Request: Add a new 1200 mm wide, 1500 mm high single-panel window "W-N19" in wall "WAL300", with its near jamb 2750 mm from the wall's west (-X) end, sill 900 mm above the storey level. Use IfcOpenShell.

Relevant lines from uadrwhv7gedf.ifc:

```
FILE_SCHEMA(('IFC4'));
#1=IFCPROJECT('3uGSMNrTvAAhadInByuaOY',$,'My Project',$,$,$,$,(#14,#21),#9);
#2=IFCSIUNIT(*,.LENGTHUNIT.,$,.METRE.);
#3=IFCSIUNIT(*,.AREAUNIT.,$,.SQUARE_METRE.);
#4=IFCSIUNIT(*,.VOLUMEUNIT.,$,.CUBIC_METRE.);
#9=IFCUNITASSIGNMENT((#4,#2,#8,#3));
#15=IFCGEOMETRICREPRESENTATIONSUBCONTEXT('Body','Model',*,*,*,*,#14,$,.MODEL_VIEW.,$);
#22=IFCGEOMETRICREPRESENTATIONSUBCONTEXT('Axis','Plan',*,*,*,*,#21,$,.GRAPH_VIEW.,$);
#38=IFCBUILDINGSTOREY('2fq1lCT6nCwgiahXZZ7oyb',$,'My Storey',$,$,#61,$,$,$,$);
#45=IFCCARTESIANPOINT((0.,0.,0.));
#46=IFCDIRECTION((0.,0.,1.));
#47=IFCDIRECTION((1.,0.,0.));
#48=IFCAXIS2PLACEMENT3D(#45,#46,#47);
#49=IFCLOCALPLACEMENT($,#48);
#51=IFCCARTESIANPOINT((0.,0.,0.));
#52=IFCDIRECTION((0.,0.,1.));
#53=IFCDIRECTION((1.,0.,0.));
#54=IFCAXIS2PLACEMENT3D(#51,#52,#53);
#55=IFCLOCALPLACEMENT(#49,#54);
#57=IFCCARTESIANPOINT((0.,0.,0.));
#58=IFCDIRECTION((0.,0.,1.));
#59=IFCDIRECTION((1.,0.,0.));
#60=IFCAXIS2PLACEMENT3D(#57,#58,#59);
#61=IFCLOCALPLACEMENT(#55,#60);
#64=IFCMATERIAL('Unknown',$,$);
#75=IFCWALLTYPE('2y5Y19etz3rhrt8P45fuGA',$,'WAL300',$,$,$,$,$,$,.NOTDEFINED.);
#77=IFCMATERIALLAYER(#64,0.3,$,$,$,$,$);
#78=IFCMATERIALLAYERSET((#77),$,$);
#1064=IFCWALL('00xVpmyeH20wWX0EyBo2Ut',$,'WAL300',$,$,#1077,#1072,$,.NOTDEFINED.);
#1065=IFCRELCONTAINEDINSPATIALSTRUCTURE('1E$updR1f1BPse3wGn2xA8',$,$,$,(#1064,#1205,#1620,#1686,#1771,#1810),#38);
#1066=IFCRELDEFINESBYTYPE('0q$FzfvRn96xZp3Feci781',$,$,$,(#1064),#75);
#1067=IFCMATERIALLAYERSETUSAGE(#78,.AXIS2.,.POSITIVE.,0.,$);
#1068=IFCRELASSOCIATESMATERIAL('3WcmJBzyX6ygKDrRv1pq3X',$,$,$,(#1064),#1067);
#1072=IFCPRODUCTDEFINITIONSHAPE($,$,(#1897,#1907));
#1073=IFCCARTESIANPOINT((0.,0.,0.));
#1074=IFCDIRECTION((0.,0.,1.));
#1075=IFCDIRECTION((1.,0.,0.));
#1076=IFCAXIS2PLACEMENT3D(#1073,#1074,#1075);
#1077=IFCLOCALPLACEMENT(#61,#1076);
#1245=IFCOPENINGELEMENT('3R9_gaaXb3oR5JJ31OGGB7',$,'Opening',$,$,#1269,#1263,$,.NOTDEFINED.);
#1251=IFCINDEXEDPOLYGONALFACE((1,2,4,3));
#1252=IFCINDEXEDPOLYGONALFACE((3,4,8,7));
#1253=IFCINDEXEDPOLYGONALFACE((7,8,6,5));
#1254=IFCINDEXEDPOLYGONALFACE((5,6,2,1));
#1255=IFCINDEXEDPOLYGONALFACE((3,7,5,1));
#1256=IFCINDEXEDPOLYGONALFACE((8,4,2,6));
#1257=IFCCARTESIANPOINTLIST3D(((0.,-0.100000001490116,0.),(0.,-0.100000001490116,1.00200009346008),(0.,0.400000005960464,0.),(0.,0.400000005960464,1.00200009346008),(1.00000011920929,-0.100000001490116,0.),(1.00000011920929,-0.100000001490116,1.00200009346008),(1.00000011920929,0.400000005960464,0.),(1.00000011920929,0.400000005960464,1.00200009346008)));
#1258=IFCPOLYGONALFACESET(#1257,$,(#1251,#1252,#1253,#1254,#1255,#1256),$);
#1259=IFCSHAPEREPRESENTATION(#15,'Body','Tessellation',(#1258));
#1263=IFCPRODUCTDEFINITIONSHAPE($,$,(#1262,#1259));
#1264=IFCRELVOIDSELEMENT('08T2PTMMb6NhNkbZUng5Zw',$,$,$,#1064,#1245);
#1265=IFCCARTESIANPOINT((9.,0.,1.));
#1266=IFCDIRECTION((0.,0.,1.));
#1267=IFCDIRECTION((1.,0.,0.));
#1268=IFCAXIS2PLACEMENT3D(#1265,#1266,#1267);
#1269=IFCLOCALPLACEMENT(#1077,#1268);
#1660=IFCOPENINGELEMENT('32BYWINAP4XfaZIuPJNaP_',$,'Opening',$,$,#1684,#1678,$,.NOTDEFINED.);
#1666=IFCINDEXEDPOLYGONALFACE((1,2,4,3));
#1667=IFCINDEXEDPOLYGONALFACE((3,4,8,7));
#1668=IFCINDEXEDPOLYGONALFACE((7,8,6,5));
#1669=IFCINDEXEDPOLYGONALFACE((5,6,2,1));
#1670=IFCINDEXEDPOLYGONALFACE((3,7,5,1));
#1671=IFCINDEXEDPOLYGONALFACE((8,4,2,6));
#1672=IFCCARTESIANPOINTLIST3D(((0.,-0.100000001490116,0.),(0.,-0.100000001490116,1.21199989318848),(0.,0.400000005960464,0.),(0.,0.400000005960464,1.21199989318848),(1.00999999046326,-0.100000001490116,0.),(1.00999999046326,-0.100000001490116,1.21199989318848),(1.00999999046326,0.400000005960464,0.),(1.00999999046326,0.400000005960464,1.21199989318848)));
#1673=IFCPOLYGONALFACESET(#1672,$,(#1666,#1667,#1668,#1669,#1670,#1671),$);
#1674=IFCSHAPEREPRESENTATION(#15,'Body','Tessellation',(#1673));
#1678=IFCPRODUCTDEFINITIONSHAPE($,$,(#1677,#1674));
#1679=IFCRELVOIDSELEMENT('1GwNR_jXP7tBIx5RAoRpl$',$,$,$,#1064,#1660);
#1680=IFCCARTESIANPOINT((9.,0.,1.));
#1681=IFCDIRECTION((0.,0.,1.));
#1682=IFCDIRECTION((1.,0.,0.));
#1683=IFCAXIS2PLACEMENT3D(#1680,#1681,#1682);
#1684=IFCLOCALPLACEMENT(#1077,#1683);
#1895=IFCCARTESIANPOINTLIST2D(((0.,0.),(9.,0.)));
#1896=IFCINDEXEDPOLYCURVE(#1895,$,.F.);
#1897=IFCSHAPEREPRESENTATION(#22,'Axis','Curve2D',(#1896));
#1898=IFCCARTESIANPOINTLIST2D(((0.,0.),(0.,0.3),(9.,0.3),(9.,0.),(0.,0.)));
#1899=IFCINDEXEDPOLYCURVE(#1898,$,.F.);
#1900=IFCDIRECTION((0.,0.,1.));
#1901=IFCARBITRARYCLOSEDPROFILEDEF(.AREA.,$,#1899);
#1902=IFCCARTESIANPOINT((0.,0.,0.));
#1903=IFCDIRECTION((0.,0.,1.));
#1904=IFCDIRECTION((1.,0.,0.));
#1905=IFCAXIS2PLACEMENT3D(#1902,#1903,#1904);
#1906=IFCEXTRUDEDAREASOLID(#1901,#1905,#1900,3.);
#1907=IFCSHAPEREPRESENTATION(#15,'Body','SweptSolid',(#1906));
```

```python
import numpy as np
import ifcopenshell
import ifcopenshell.api.feature
import ifcopenshell.api.geometry
import ifcopenshell.api.root
import ifcopenshell.api.spatial
import ifcopenshell.geom
import ifcopenshell.util.element
import ifcopenshell.util.placement
import ifcopenshell.util.representation
import ifcopenshell.util.shape
import ifcopenshell.util.unit

model = ifcopenshell.open("uadrwhv7gedf.ifc")
unit_scale = ifcopenshell.util.unit.calculate_unit_scale(model)
settings = ifcopenshell.geom.settings()


def volume(element):
    """Net volume in cubic metres, openings subtracted."""
    shape = ifcopenshell.geom.create_shape(settings, element)
    return ifcopenshell.util.shape.get_volume(shape.geometry)


wall = model.by_guid("00xVpmyeH20wWX0EyBo2Ut")
storey = ifcopenshell.util.element.get_container(wall, ifc_class="IfcBuildingStorey")
context = ifcopenshell.util.representation.get_context(model, "Model", "Body", "MODEL_VIEW")
before = volume(wall)

width, height, from_end, sill = 1.2, 1.5, 2.75, 0.9  # metres

# The wall runs along its own X axis, and the end named is its -X end.
wall_shape = ifcopenshell.geom.create_shape(settings, wall)
x, y, z = ifcopenshell.util.shape.get_vertices(wall_shape.geometry).T
start = x.min() + from_end
face, thickness = float(y.min()), float(y.max() - y.min())
wall_matrix = ifcopenshell.util.placement.get_local_placement(wall.ObjectPlacement)
level = ifcopenshell.util.placement.get_local_placement(storey.ObjectPlacement)[2, 3]


def in_wall(x, y):
    """Placement at x, y metres in the wall's axes, at sill height."""
    matrix = wall_matrix.copy()
    matrix[:, 3] = wall_matrix @ np.array([x / unit_scale, y / unit_scale, 0.0, 1.0])
    matrix[2, 3] = level + sill / unit_scale
    return matrix


# Opening: a box that overshoots both wall faces by 50 mm.
opening = ifcopenshell.api.root.create_entity(model, ifc_class="IfcOpeningElement", predefined_type="OPENING")
box = ifcopenshell.api.geometry.add_wall_representation(
    model, context=context, length=width, height=height, thickness=thickness + 0.1
)
ifcopenshell.api.geometry.assign_representation(model, product=opening, representation=box)
ifcopenshell.api.geometry.edit_object_placement(model, product=opening, matrix=in_wall(start, face - 0.05), is_si=False)
ifcopenshell.api.feature.add_feature(model, feature=opening, element=wall)

window = ifcopenshell.api.root.create_entity(model, ifc_class="IfcWindow", name="W-N19", predefined_type="WINDOW")
window.OverallWidth, window.OverallHeight = width / unit_scale, height / unit_scale
window.PartitioningType = "SINGLE_PANEL"
body = ifcopenshell.api.geometry.add_window_representation(
    model,
    context=context,
    overall_width=window.OverallWidth,
    overall_height=window.OverallHeight,
    partition_type="SINGLE_PANEL",
)
ifcopenshell.api.geometry.assign_representation(model, product=window, representation=body)
ifcopenshell.api.spatial.assign_container(model, products=[window], relating_structure=storey)
ifcopenshell.api.feature.add_filling(model, opening=opening, element=window)

# Centre the window in the wall's thickness.
ifcopenshell.api.geometry.edit_object_placement(model, product=window, matrix=in_wall(start, face), is_si=False)
window_shape = ifcopenshell.geom.create_shape(settings, window)
depth = ifcopenshell.util.shape.get_vertices(window_shape.geometry)[:, 1]
offset = face + thickness / 2 - (depth.min() + depth.max()) / 2
ifcopenshell.api.geometry.edit_object_placement(model, product=window, matrix=in_wall(start, offset), is_si=False)

after = volume(wall)

print(f"wall volume {before:.3f} -> {after:.3f} m3")

model.write("uadrwhv7gedf-out.ifc")
```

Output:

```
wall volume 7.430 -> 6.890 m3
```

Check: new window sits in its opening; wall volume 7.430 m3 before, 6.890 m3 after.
